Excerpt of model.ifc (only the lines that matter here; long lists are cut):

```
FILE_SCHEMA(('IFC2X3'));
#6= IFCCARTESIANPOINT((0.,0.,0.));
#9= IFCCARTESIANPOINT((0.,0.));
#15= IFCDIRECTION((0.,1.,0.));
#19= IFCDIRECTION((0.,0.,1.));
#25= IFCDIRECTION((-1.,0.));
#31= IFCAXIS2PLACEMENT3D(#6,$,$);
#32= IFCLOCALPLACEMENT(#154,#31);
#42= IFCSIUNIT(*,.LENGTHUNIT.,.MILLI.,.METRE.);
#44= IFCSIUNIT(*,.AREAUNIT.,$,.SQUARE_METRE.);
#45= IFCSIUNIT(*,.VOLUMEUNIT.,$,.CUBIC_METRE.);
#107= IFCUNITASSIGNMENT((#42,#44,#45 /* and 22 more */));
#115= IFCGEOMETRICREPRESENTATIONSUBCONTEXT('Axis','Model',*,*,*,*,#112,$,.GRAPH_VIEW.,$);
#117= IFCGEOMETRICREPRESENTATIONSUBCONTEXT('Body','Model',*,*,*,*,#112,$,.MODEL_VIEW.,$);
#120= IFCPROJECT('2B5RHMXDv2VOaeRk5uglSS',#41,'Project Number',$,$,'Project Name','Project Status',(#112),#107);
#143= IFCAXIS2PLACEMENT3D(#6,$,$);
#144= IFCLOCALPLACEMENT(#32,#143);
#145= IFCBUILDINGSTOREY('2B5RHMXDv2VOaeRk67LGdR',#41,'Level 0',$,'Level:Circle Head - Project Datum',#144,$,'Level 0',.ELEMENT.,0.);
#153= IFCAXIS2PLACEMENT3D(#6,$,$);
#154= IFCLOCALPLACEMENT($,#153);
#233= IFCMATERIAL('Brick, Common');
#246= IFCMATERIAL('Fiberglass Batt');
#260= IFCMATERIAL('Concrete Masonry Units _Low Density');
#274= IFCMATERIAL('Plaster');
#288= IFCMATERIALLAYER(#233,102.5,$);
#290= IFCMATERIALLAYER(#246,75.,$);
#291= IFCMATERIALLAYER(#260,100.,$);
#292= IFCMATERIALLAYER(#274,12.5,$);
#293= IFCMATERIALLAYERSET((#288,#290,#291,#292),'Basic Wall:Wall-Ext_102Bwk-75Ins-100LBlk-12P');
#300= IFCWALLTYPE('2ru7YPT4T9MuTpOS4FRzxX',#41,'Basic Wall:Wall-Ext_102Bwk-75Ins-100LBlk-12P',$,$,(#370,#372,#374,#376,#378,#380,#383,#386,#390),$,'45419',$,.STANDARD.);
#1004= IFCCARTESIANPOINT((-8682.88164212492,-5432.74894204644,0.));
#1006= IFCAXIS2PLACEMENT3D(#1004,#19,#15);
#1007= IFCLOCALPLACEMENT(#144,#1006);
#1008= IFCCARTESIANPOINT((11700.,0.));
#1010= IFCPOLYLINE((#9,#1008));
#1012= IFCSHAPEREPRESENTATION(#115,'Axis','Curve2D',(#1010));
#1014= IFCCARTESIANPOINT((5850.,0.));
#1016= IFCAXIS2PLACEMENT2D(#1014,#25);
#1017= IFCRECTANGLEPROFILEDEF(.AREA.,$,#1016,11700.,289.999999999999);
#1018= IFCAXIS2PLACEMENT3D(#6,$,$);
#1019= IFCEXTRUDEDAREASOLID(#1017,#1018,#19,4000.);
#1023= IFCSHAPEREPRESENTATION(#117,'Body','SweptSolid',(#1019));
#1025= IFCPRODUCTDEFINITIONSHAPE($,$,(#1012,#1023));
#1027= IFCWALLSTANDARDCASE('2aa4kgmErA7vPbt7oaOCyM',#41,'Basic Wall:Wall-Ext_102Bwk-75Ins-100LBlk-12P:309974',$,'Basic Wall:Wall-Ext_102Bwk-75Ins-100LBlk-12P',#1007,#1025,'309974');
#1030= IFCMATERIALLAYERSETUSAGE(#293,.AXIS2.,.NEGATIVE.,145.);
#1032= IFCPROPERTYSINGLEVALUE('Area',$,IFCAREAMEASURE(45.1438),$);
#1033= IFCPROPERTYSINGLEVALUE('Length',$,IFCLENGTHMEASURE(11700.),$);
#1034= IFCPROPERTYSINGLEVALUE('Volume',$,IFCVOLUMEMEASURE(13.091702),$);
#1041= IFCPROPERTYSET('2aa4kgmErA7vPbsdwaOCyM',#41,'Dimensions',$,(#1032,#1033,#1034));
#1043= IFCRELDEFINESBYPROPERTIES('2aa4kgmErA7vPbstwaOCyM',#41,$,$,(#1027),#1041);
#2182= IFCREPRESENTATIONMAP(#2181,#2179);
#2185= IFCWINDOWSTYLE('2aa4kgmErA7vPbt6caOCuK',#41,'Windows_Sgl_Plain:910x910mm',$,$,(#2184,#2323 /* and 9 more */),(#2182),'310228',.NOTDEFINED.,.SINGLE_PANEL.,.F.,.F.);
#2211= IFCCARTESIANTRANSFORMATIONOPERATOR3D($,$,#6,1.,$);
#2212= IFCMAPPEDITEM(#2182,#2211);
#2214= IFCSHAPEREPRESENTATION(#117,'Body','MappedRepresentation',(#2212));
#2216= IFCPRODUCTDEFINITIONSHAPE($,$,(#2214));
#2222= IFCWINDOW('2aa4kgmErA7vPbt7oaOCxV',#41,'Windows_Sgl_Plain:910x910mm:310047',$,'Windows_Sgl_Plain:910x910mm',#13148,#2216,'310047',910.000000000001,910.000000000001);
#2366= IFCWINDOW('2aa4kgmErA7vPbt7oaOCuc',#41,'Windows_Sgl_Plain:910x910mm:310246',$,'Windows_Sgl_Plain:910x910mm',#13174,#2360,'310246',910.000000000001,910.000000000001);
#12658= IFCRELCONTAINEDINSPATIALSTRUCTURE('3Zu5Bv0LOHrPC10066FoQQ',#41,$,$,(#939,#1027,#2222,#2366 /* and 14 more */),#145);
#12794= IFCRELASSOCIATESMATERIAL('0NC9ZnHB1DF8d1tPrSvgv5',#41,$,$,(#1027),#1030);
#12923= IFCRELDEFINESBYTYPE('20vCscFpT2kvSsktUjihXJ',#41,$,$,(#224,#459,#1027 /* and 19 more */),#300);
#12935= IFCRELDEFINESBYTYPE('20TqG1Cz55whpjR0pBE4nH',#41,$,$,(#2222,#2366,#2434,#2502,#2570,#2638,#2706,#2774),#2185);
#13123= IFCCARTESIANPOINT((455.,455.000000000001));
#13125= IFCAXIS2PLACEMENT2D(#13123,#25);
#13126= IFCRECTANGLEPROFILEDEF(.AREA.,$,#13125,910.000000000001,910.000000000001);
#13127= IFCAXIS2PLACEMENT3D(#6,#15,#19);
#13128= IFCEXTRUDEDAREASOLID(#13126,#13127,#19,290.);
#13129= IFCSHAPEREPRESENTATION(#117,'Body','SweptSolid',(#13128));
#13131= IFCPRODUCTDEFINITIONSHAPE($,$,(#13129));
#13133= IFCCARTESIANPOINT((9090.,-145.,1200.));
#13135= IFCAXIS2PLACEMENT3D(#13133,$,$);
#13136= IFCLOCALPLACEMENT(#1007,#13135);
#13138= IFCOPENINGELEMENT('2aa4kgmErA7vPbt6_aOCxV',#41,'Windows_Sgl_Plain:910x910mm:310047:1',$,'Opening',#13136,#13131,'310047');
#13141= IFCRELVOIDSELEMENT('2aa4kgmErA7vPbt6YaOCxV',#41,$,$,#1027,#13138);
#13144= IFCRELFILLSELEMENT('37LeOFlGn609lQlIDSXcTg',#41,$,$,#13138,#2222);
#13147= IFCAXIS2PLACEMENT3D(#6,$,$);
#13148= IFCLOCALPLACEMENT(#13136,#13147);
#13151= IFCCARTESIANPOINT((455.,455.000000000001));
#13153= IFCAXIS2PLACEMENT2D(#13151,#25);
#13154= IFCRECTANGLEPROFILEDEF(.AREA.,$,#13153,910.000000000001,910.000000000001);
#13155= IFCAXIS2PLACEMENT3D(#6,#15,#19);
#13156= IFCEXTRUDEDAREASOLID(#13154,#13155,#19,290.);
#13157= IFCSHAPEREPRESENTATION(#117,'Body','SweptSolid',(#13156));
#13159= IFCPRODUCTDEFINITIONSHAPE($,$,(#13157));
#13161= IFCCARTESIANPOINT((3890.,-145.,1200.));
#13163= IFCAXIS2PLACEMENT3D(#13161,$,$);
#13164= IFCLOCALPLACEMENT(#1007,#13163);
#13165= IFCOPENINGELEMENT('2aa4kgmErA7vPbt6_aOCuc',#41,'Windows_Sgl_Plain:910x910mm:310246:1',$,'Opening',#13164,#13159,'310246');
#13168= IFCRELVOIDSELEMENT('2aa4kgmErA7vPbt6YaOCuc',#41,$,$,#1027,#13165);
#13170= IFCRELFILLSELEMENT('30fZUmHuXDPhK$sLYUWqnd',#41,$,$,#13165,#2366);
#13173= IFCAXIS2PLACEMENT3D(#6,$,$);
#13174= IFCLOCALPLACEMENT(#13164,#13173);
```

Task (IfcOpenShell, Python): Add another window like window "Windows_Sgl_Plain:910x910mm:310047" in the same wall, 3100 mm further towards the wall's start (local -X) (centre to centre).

```python
import ifcopenshell
import ifcopenshell.api.feature
import ifcopenshell.api.geometry
import ifcopenshell.api.pset
import ifcopenshell.api.root
import ifcopenshell.geom
import ifcopenshell.util.element
import ifcopenshell.util.placement
import ifcopenshell.util.shape
import ifcopenshell.util.unit

model = ifcopenshell.open("model.ifc")
unit_scale = ifcopenshell.util.unit.calculate_unit_scale(model)
area_scale = ifcopenshell.util.unit.calculate_unit_scale(model, "AREAUNIT")
volume_scale = ifcopenshell.util.unit.calculate_unit_scale(model, "VOLUMEUNIT")
settings = ifcopenshell.geom.settings()


def volume(element):
    """Net volume in cubic metres, openings subtracted."""
    shape = ifcopenshell.geom.create_shape(settings, element)
    return ifcopenshell.util.shape.get_volume(shape.geometry)


def reuse_history(source, copy):
    """copy_class also copies each property set's owner history, people and application; keep the originals."""
    for rel in copy.IsDefinedBy:
        if rel.is_a("IfcRelDefinesByProperties") and (history := rel.RelatingPropertyDefinition.OwnerHistory):
            rel.RelatingPropertyDefinition.OwnerHistory = source.OwnerHistory
            ifcopenshell.util.element.remove_deep2(model, history)


window = model.by_guid("2aa4kgmErA7vPbt7oaOCxV")
opening = window.FillsVoids[0].RelatingOpeningElement
wall = opening.VoidsElements[0].RelatingBuildingElement
before = volume(wall)
shift = ifcopenshell.util.placement.get_local_placement(wall.ObjectPlacement)[:3, 0] * -3.1 / unit_scale

# copy_class copies the void relationship, type, container and properties, but no geometry.
new_opening = ifcopenshell.api.root.copy_class(model, product=opening)
new_opening.Representation = ifcopenshell.util.element.copy_deep(
    model, opening.Representation, exclude=["IfcGeometricRepresentationContext", "IfcRepresentationMap"]
)
new_opening.Name = "Windows_Sgl_Plain:910x910mm"
new_opening.Tag = None
new_window = ifcopenshell.api.root.copy_class(model, product=window)
new_window.Representation = ifcopenshell.util.element.copy_deep(
    model, window.Representation, exclude=["IfcGeometricRepresentationContext", "IfcRepresentationMap"]
)
new_window.Name = "Windows_Sgl_Plain:910x910mm"
new_window.Tag = None
reuse_history(window, new_window)
fills = ifcopenshell.api.feature.add_filling(model, opening=new_opening, element=new_window)
fills.OwnerHistory = new_window.OwnerHistory  # required in IFC2X3

for old, new in ((opening, new_opening), (window, new_window)):
    matrix = ifcopenshell.util.placement.get_local_placement(old.ObjectPlacement)
    matrix[:3, 3] += shift
    ifcopenshell.api.geometry.edit_object_placement(model, product=new, matrix=matrix, is_si=False)

after = volume(wall)
thickness = 0.29  # wall thickness in metres

# Update the wall's stored quantities.
pset = model.by_id(ifcopenshell.util.element.get_pset(wall, "Dimensions", should_inherit=False)["id"])
ifcopenshell.api.pset.edit_pset(model, pset=pset, properties={
    "Area": model.create_entity("IfcAreaMeasure", after / thickness / area_scale),
    "Volume": model.create_entity("IfcVolumeMeasure", after / volume_scale),
})

print(f"wall volume {before:.3f} -> {after:.3f} m3")

model.write("model_edited.ifc")
```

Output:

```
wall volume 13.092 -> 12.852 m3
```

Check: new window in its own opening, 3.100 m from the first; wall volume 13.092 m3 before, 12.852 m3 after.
